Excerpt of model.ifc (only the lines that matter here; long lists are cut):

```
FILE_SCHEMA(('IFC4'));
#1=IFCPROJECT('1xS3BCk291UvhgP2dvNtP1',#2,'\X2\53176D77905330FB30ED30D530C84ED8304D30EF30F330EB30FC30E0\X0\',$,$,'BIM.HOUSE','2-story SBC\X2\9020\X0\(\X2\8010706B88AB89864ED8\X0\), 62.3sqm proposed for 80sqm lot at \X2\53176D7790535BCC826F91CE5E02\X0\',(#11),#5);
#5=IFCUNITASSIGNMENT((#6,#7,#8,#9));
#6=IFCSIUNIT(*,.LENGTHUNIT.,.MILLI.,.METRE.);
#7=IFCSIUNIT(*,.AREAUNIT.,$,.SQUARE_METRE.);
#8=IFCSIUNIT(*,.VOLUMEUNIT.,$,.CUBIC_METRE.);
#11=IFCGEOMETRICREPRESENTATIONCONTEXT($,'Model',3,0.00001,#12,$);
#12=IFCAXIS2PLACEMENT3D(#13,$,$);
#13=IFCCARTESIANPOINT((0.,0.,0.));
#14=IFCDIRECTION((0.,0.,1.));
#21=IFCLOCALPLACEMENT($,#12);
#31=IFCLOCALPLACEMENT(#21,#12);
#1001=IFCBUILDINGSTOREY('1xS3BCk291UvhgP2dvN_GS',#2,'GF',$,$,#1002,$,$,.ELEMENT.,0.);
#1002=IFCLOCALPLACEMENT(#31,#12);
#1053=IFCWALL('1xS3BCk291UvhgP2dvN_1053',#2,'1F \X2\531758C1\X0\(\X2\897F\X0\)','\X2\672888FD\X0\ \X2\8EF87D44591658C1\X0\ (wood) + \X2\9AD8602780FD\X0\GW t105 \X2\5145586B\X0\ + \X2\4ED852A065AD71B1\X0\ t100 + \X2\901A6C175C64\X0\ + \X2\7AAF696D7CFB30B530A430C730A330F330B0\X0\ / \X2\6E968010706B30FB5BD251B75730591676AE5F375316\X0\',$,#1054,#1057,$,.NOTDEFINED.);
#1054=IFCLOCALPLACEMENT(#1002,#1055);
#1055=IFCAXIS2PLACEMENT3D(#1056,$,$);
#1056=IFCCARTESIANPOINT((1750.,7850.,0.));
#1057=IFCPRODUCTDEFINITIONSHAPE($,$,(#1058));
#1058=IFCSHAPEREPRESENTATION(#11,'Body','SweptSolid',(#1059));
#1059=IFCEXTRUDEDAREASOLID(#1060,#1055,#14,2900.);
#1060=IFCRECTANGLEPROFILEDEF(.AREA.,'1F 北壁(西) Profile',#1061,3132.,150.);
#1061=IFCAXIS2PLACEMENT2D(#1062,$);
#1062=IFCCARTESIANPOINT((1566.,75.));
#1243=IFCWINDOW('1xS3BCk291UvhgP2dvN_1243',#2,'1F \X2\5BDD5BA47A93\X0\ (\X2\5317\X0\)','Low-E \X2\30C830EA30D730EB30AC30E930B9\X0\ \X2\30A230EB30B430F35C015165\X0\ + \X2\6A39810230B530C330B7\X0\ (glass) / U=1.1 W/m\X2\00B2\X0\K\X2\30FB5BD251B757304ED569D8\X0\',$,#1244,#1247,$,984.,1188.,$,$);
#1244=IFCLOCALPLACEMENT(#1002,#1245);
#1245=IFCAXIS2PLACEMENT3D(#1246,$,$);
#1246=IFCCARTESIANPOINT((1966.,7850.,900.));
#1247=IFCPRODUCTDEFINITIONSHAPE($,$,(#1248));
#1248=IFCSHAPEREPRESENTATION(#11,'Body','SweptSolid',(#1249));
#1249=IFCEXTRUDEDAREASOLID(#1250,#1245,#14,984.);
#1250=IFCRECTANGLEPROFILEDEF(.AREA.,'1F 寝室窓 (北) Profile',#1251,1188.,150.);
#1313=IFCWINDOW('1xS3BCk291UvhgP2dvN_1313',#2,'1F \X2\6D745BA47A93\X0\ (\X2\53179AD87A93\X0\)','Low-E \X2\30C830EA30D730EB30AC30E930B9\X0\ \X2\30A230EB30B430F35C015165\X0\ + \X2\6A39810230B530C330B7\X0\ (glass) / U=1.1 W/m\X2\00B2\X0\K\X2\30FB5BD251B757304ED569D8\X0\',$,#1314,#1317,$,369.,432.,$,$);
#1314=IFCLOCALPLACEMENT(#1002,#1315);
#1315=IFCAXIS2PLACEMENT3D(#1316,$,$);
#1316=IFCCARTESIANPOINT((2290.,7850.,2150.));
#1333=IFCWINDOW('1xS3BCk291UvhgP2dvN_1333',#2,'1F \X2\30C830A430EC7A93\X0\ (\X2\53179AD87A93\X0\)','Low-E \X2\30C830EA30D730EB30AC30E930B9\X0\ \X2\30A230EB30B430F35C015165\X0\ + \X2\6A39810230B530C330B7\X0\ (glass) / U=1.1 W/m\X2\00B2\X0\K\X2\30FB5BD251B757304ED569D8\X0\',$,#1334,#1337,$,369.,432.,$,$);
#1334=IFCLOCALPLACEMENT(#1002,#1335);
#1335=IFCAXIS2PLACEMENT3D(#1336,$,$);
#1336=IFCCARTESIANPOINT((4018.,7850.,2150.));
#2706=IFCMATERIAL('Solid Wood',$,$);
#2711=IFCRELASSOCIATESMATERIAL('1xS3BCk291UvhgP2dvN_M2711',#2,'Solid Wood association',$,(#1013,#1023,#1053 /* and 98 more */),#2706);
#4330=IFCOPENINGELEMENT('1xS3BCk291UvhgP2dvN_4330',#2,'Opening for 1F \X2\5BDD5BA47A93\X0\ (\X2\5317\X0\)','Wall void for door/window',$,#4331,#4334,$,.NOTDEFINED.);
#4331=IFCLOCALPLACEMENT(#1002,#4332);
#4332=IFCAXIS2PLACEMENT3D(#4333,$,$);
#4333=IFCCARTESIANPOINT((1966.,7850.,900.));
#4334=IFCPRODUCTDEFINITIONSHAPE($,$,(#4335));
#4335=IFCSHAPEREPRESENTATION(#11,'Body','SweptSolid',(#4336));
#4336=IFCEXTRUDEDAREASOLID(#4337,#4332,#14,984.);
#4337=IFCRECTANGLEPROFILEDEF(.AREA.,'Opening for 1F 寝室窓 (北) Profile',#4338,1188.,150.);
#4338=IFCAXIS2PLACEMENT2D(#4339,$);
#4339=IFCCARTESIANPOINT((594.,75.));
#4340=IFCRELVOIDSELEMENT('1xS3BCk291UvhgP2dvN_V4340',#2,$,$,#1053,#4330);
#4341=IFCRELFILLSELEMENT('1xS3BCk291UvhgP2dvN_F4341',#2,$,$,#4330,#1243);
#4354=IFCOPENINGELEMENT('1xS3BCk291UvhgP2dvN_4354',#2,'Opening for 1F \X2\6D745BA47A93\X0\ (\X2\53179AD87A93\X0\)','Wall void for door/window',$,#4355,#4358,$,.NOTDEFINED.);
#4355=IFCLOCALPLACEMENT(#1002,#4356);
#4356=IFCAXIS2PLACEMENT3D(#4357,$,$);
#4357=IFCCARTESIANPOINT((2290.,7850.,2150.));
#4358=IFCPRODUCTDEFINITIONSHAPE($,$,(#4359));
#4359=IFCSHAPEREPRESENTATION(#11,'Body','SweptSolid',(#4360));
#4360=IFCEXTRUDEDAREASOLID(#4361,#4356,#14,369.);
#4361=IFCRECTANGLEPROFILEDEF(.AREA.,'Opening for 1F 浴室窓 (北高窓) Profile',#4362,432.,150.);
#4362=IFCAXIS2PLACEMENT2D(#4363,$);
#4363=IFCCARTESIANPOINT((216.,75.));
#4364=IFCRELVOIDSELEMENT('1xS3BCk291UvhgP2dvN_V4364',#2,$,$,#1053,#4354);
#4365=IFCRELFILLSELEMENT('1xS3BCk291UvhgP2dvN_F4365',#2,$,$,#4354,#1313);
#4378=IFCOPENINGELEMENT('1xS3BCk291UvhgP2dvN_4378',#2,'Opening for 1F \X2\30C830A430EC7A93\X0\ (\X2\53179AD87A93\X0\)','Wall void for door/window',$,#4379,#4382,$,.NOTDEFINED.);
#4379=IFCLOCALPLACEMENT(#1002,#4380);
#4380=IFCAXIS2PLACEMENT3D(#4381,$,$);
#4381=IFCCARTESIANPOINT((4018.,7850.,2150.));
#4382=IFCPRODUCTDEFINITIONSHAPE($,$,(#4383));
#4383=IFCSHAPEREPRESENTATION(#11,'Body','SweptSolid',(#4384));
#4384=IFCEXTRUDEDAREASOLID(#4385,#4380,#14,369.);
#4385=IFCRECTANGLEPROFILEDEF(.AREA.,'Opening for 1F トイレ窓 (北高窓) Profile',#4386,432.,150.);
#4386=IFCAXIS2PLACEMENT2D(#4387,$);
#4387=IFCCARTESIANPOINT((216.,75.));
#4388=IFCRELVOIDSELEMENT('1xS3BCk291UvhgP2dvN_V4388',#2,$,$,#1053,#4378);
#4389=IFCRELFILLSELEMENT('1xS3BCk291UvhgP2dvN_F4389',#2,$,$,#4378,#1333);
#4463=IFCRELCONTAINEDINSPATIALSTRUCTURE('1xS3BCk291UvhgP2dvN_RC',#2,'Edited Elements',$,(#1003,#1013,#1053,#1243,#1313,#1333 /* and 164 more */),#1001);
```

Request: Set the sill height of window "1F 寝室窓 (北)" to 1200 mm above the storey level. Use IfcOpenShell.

```python
import numpy as np
import ifcopenshell
import ifcopenshell.api.geometry
import ifcopenshell.geom
import ifcopenshell.util.element
import ifcopenshell.util.placement
import ifcopenshell.util.shape
import ifcopenshell.util.unit

model = ifcopenshell.open("model.ifc")
unit_scale = ifcopenshell.util.unit.calculate_unit_scale(model)

window = model.by_guid("1xS3BCk291UvhgP2dvN_1243")
opening = window.FillsVoids[0].RelatingOpeningElement
storey = ifcopenshell.util.element.get_container(window, ifc_class="IfcBuildingStorey")
level = ifcopenshell.util.placement.get_local_placement(storey.ObjectPlacement)[2, 3]

# The opening's origin need not be at the sill, so measure its lowest point.
shape = ifcopenshell.geom.create_shape(ifcopenshell.geom.settings(), opening)
bottom = ifcopenshell.util.shape.get_shape_bottom_elevation(shape, shape.geometry) / unit_scale
dz = level + 1200.0 - bottom

shift = np.array([0.0, 0.0, dz])
# The window is not placed relative to its opening, so move both.
for product in (opening, window):
    matrix = ifcopenshell.util.placement.get_local_placement(product.ObjectPlacement)
    matrix[:3, 3] += shift
    ifcopenshell.api.geometry.edit_object_placement(model, product=product, matrix=matrix, is_si=False)

print(f"moved by {dz * unit_scale:+.3f} m")

model.write("model-out.ifc")
```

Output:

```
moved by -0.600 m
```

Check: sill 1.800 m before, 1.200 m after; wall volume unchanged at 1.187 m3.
